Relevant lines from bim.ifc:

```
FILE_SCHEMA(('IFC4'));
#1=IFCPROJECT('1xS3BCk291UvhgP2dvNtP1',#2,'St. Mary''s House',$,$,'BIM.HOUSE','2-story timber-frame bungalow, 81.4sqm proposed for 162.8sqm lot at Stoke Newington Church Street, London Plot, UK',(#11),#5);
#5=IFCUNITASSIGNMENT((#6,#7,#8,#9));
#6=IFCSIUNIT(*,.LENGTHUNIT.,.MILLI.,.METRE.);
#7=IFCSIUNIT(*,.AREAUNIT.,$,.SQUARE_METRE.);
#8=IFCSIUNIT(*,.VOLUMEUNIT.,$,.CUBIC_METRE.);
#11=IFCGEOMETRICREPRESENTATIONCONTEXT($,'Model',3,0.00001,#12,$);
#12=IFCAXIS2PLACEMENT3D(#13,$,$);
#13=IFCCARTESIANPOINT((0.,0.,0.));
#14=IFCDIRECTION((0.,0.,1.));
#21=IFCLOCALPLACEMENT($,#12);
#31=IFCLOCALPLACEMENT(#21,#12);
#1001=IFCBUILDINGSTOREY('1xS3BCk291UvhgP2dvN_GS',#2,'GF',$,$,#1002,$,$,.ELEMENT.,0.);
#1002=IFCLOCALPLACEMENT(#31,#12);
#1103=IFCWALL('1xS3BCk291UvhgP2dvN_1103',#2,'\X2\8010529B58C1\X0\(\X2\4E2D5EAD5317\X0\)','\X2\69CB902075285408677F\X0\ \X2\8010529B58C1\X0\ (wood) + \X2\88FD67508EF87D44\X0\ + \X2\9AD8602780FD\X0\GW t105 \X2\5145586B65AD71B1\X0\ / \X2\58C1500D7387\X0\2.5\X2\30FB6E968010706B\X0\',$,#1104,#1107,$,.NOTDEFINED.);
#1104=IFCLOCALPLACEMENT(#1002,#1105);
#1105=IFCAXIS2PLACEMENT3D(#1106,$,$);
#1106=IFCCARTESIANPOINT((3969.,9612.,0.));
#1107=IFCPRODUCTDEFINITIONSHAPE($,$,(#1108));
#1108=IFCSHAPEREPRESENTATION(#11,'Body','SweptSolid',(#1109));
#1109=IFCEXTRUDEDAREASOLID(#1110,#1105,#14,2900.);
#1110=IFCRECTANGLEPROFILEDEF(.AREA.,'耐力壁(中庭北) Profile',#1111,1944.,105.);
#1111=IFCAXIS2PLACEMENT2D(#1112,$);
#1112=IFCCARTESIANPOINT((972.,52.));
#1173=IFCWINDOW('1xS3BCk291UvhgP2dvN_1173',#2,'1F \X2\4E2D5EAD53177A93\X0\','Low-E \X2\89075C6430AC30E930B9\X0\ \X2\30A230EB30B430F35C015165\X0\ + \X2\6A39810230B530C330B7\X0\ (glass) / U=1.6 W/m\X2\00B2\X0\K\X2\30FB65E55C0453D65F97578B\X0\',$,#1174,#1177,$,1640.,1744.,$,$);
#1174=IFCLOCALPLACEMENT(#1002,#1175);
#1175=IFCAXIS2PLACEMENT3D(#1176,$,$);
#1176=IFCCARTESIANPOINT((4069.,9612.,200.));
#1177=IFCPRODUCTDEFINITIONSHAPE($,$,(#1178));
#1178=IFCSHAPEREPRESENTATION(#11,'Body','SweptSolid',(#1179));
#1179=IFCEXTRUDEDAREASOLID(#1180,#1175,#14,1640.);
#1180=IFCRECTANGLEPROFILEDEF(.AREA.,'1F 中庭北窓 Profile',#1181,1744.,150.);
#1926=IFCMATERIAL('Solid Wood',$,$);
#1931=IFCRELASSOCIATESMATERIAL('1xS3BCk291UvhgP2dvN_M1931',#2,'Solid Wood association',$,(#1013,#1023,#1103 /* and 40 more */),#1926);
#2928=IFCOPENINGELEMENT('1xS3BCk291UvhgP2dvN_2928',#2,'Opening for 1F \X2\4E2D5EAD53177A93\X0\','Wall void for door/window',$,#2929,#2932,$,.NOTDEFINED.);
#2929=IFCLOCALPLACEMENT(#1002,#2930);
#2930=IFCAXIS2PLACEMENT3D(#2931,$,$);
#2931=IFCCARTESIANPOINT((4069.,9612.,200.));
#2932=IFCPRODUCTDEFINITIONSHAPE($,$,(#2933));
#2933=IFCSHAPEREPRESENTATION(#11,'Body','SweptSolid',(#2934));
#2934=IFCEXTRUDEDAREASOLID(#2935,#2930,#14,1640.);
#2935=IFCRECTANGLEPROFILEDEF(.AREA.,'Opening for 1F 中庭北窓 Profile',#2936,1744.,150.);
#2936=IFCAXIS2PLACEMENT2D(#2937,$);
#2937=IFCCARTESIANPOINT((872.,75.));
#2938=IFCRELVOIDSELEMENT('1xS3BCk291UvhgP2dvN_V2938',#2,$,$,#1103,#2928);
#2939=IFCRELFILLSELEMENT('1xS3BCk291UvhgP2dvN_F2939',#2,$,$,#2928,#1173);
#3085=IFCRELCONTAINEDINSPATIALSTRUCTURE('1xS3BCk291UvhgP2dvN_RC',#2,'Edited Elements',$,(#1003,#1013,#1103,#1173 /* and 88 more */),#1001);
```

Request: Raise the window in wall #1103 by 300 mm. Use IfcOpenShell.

```python
import numpy as np
import ifcopenshell
import ifcopenshell.api.geometry
import ifcopenshell.util.placement
import ifcopenshell.util.unit

model = ifcopenshell.open("bim.ifc")
unit_scale = ifcopenshell.util.unit.calculate_unit_scale(model)

window = model.by_guid("1xS3BCk291UvhgP2dvN_1173")
opening = window.FillsVoids[0].RelatingOpeningElement
dz = 300.0

shift = np.array([0.0, 0.0, dz])
# The window is not placed relative to its opening, so move both.
for product in (opening, window):
    matrix = ifcopenshell.util.placement.get_local_placement(product.ObjectPlacement)
    matrix[:3, 3] += shift
    ifcopenshell.api.geometry.edit_object_placement(model, product=product, matrix=matrix, is_si=False)

print(f"moved by {dz * unit_scale:+.3f} m")

model.write("bim_rev.ifc")
```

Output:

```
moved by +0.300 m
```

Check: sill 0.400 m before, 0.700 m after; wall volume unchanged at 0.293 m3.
